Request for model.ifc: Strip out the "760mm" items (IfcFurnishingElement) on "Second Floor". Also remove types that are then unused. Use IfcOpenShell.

First a look at what the model holds.

```python
import ifcopenshell
import ifcopenshell.util.element

model = ifcopenshell.open("model.ifc")
print(model.schema)
storey = next(s for s in model.by_type("IfcBuildingStorey") if s.Name == "Second Floor")
furniture = [e for e in ifcopenshell.util.element.get_decomposition(storey) if e.is_a("IfcFurnishingElement")]
seen = {}
for e in furniture:
    element_type = ifcopenshell.util.element.get_type(e)
    name = element_type.Name if element_type not in (None, e) else None
    seen[name] = seen.get(name, 0) + 1
for name, count in sorted(seen.items(), key=str):
    print(count, "x", name)
```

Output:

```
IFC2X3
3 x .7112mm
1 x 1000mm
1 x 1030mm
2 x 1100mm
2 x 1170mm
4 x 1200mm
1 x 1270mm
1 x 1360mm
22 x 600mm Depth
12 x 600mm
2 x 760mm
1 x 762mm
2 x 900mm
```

```python
import ifcopenshell
import ifcopenshell.api.root
import ifcopenshell.util.element

model = ifcopenshell.open("model.ifc")

storey = next(s for s in model.by_type("IfcBuildingStorey") if s.Name == "Second Floor")
furniture = [e for e in ifcopenshell.util.element.get_decomposition(storey) if e.is_a("IfcFurnishingElement")]
targets = [e for e in furniture if (t := ifcopenshell.util.element.get_type(e)) not in (None, e) and t.Name == "760mm"]
types = {ifcopenshell.util.element.get_type(e) for e in targets} - {None, *targets}

for e in targets:
    ifcopenshell.api.root.remove_product(model, product=e)
print(len(targets), "removed")

unused = [t for t in types if not ifcopenshell.util.element.get_types(t)]
for t in unused:
    ifcopenshell.api.root.remove_product(model, product=t)
print(len(unused), "unused types removed")

model.write("model_edited.ifc")
```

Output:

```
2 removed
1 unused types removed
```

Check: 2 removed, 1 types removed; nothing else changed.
